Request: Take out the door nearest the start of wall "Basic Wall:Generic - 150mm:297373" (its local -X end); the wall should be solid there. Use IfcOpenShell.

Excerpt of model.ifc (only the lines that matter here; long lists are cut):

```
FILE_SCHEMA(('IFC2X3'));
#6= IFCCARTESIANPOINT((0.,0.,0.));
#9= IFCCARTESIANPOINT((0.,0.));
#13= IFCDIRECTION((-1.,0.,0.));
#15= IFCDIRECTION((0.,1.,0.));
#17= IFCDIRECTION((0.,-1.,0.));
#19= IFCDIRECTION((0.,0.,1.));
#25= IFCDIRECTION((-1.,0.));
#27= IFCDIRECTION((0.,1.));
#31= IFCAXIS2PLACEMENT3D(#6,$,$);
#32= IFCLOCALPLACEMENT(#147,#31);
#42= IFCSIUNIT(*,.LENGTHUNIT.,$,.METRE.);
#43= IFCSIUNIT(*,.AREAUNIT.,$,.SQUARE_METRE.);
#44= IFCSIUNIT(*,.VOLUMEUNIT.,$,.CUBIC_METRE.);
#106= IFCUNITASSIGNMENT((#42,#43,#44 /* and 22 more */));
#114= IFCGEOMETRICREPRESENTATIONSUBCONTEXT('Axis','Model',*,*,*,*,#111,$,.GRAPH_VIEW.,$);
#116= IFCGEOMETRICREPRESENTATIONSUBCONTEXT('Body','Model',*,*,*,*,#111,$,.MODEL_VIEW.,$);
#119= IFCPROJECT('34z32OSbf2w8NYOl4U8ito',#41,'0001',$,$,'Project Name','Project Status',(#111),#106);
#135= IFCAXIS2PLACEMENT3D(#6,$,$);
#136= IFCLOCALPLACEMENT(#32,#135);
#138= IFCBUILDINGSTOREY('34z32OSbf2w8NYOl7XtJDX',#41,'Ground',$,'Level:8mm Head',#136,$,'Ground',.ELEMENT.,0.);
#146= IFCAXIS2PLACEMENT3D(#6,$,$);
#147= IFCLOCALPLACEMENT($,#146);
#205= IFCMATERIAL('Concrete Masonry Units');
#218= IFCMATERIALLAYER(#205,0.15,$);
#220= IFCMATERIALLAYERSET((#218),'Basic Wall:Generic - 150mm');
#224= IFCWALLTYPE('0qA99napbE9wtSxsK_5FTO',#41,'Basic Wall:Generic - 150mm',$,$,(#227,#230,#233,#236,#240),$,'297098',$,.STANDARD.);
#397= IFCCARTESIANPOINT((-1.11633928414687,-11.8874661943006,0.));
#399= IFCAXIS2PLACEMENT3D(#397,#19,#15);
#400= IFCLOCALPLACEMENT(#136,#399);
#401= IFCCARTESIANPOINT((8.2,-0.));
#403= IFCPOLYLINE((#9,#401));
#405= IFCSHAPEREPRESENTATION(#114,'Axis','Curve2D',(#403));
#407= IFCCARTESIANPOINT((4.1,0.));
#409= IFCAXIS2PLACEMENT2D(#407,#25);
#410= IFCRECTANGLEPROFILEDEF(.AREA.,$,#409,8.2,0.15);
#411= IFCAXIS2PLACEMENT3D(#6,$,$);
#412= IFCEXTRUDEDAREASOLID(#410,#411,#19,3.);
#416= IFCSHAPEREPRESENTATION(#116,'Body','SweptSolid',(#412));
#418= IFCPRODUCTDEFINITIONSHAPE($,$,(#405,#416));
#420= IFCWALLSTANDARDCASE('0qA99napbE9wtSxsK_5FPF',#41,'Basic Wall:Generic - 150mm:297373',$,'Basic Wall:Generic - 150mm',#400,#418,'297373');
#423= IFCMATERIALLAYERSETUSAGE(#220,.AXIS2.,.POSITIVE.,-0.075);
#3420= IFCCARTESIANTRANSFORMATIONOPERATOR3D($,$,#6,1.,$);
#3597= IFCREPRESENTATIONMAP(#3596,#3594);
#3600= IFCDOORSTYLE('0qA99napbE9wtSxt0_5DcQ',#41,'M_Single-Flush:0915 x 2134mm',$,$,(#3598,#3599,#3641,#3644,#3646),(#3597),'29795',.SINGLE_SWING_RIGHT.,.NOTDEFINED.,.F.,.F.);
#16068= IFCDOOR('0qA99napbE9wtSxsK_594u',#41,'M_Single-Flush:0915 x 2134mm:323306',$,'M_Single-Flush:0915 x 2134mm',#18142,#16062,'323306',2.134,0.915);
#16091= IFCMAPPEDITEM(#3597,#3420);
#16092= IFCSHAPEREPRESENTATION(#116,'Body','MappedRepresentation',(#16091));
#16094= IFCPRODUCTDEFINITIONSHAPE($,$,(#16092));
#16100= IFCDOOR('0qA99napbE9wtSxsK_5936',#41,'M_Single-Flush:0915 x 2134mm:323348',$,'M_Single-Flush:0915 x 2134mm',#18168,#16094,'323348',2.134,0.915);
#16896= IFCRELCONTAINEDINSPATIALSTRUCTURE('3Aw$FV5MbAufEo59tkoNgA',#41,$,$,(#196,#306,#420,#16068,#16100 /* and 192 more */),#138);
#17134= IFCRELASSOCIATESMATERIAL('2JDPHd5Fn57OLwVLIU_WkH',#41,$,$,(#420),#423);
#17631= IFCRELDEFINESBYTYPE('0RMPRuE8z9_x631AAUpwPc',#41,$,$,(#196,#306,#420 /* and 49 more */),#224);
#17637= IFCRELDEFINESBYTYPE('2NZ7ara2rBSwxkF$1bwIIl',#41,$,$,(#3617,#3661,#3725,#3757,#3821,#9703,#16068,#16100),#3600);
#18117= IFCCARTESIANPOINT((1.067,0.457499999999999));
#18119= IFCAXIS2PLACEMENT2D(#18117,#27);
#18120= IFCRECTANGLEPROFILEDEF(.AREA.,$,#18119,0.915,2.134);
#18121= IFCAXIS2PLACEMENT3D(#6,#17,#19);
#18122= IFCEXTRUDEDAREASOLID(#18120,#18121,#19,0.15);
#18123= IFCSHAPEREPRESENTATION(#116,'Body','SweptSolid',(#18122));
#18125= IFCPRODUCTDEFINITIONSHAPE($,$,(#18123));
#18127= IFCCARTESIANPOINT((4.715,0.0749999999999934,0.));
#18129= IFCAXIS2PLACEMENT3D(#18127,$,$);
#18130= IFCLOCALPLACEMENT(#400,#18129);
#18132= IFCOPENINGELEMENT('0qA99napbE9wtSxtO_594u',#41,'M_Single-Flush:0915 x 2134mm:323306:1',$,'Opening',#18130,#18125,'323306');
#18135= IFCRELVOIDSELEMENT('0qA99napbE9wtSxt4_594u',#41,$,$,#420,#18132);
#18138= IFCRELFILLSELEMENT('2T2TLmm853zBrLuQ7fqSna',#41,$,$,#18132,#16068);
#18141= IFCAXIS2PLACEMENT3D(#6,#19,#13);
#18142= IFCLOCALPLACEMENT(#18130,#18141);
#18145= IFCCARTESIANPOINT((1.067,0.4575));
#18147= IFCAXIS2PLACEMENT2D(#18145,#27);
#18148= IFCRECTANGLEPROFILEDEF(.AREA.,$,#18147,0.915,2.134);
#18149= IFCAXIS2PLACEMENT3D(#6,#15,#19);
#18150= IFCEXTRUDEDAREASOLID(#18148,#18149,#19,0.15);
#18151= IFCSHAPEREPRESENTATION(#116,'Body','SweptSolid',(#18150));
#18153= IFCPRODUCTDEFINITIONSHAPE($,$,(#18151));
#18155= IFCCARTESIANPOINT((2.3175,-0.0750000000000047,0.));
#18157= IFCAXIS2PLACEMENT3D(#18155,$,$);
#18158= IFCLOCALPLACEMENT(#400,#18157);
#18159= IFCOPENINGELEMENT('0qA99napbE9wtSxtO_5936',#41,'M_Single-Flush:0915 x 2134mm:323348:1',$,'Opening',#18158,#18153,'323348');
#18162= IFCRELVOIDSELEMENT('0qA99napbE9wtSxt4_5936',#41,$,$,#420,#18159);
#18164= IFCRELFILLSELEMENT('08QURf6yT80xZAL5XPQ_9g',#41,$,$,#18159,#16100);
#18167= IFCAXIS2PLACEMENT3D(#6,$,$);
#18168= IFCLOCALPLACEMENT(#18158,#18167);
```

```python
import ifcopenshell
import ifcopenshell.api.feature
import ifcopenshell.api.root
import ifcopenshell.geom
import ifcopenshell.util.shape

model = ifcopenshell.open("model.ifc")
settings = ifcopenshell.geom.settings()


def volume(element):
    """Net volume in cubic metres, openings subtracted."""
    shape = ifcopenshell.geom.create_shape(settings, element)
    return ifcopenshell.util.shape.get_volume(shape.geometry)


door = model.by_id(16100)
opening = door.FillsVoids[0].RelatingOpeningElement
wall = opening.VoidsElements[0].RelatingBuildingElement
before = volume(wall)

ifcopenshell.api.root.remove_product(model, product=door)
ifcopenshell.api.feature.remove_feature(model, feature=opening)

after = volume(wall)

print(f"wall volume {before:.3f} -> {after:.3f} m3")

model.write("model_edited.ifc")
```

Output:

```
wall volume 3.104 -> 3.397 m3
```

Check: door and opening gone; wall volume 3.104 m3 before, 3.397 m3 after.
